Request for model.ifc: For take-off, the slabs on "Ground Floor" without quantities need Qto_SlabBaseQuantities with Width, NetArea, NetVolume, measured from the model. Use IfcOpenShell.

First a look at what the model holds.

```python
import ifcopenshell
import ifcopenshell.util.element
import ifcopenshell.util.unit

model = ifcopenshell.open("model.ifc")
print(model.schema)
for unit_type in ("LENGTHUNIT", "AREAUNIT", "VOLUMEUNIT"):
    print(unit_type, ifcopenshell.util.unit.calculate_unit_scale(model, unit_type))
storey = next(s for s in model.by_type("IfcBuildingStorey") if s.Name == "Ground Floor")
slabs = [e for e in ifcopenshell.util.element.get_decomposition(storey) if e.is_a("IfcSlab")]
for e in sorted(slabs, key=lambda e: e.id()):
    print(e.id(), e.is_a(), e.Name, list(ifcopenshell.util.element.get_psets(e, qtos_only=True)), sep=" | ")
```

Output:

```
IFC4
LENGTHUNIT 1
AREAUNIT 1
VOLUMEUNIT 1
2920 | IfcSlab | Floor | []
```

```python
import ifcopenshell
import ifcopenshell.api.pset
import ifcopenshell.geom
import ifcopenshell.util.element
import ifcopenshell.util.shape
import ifcopenshell.util.unit

model = ifcopenshell.open("model.ifc")
unit_scale = ifcopenshell.util.unit.calculate_unit_scale(model)
area_scale = ifcopenshell.util.unit.calculate_unit_scale(model, "AREAUNIT")
volume_scale = ifcopenshell.util.unit.calculate_unit_scale(model, "VOLUMEUNIT")
settings = ifcopenshell.geom.settings()

storey = next(s for s in model.by_type("IfcBuildingStorey") if s.Name == "Ground Floor")
slabs = [e for e in ifcopenshell.util.element.get_decomposition(storey) if e.is_a("IfcSlab")]

for e in sorted(slabs, key=lambda e: e.id()):
    if ifcopenshell.util.element.get_psets(e, qtos_only=True, should_inherit=False):
        continue
    # Geometry comes back in metres, in the element's own axes.
    shape = ifcopenshell.geom.create_shape(settings, e)
    values = {
        "Width": ifcopenshell.util.shape.get_z(shape.geometry) / unit_scale,
        "NetArea": ifcopenshell.util.shape.get_footprint_area(shape.geometry) / area_scale,
        "NetVolume": ifcopenshell.util.shape.get_volume(shape.geometry) / volume_scale,
    }
    qto = ifcopenshell.api.pset.add_qto(model, product=e, name="Qto_SlabBaseQuantities")
    ifcopenshell.api.pset.edit_qto(model, qto=qto, properties=values)
    print(e.id(), {k: round(v, 3) for k, v in values.items()})

model.write("model_edited.ifc")
```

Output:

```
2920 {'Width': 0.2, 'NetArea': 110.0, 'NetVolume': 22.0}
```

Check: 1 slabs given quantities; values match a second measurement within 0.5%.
